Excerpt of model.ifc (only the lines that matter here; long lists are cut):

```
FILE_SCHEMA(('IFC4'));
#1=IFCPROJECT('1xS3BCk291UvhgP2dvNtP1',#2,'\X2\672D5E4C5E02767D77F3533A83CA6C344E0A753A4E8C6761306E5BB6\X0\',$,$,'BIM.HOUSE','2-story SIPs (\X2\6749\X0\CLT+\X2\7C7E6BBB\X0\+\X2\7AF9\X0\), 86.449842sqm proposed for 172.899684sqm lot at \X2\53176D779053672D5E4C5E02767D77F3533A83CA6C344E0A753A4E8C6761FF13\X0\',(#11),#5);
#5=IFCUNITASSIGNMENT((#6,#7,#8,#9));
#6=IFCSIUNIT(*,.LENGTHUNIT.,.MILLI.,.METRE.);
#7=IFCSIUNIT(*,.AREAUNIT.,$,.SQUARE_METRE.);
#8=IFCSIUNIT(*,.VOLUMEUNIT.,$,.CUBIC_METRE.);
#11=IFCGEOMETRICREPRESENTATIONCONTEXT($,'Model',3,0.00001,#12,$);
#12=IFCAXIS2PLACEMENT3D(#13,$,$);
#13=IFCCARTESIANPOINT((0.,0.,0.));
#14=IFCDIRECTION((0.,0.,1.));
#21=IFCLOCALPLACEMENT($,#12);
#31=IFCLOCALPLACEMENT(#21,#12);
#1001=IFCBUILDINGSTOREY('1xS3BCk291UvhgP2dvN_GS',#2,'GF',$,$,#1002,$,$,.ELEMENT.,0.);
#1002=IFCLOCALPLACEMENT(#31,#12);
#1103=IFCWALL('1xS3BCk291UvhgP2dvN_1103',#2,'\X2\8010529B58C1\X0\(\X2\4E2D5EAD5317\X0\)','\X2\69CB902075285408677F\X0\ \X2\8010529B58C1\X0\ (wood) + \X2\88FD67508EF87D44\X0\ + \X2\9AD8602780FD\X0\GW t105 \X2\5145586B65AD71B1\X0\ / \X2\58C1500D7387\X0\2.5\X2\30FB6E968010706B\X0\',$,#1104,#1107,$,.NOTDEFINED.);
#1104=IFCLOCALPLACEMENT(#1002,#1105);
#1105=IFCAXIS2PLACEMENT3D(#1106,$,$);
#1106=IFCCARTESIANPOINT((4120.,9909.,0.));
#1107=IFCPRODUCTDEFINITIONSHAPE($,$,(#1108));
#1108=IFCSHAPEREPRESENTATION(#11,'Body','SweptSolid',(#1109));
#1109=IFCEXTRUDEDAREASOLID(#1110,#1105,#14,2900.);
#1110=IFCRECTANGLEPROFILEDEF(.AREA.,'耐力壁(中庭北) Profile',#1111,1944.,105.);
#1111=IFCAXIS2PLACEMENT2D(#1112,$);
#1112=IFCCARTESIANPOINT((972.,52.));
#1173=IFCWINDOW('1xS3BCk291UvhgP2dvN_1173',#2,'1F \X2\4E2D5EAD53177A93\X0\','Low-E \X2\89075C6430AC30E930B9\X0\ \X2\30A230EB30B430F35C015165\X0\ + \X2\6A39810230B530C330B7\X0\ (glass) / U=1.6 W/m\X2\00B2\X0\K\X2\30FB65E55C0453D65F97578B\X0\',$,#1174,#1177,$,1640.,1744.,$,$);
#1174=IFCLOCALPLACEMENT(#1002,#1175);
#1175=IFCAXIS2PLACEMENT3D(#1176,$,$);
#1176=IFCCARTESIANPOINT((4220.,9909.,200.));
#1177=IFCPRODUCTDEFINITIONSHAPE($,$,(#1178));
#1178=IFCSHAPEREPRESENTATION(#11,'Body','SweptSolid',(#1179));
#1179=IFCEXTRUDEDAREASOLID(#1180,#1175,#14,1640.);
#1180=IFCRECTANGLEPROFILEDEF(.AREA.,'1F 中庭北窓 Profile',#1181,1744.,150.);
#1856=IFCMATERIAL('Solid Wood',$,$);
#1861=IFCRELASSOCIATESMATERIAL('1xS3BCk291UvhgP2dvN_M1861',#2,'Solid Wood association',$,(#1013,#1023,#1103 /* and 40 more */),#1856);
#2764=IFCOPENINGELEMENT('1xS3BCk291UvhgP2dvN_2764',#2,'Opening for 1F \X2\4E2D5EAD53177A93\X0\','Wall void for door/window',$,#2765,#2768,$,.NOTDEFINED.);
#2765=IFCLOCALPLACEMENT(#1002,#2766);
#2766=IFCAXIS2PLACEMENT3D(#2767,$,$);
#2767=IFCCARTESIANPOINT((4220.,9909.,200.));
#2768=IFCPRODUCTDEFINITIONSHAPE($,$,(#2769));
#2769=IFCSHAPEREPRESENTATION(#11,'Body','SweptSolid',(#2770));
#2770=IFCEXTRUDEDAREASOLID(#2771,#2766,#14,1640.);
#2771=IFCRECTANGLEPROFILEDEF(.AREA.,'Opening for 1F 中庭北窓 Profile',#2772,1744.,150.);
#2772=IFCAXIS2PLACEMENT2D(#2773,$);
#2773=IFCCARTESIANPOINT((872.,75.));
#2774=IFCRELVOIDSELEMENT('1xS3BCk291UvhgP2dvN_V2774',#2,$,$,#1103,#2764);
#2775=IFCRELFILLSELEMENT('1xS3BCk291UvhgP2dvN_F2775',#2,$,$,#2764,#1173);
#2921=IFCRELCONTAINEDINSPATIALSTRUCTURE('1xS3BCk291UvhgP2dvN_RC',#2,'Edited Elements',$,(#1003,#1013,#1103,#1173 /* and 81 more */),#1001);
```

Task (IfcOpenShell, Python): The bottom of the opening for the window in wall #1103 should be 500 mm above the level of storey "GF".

```python
import numpy as np
import ifcopenshell
import ifcopenshell.api.geometry
import ifcopenshell.geom
import ifcopenshell.util.element
import ifcopenshell.util.placement
import ifcopenshell.util.shape
import ifcopenshell.util.unit

model = ifcopenshell.open("model.ifc")
unit_scale = ifcopenshell.util.unit.calculate_unit_scale(model)

window = model.by_id(1173)
opening = window.FillsVoids[0].RelatingOpeningElement
storey = ifcopenshell.util.element.get_container(window, ifc_class="IfcBuildingStorey")
level = ifcopenshell.util.placement.get_local_placement(storey.ObjectPlacement)[2, 3]

# The opening's origin need not be at the sill, so measure its lowest point.
shape = ifcopenshell.geom.create_shape(ifcopenshell.geom.settings(), opening)
bottom = ifcopenshell.util.shape.get_shape_bottom_elevation(shape, shape.geometry) / unit_scale
dz = level + 0.5 / unit_scale - bottom

shift = np.array([0.0, 0.0, dz])
# The window is not placed relative to its opening, so move both.
for product in (opening, window):
    matrix = ifcopenshell.util.placement.get_local_placement(product.ObjectPlacement)
    matrix[:3, 3] += shift
    ifcopenshell.api.geometry.edit_object_placement(model, product=product, matrix=matrix, is_si=False)

print(f"moved by {dz * unit_scale:+.3f} m")

model.write("model-out.ifc")
```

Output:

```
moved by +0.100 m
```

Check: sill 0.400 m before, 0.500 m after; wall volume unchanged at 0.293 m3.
